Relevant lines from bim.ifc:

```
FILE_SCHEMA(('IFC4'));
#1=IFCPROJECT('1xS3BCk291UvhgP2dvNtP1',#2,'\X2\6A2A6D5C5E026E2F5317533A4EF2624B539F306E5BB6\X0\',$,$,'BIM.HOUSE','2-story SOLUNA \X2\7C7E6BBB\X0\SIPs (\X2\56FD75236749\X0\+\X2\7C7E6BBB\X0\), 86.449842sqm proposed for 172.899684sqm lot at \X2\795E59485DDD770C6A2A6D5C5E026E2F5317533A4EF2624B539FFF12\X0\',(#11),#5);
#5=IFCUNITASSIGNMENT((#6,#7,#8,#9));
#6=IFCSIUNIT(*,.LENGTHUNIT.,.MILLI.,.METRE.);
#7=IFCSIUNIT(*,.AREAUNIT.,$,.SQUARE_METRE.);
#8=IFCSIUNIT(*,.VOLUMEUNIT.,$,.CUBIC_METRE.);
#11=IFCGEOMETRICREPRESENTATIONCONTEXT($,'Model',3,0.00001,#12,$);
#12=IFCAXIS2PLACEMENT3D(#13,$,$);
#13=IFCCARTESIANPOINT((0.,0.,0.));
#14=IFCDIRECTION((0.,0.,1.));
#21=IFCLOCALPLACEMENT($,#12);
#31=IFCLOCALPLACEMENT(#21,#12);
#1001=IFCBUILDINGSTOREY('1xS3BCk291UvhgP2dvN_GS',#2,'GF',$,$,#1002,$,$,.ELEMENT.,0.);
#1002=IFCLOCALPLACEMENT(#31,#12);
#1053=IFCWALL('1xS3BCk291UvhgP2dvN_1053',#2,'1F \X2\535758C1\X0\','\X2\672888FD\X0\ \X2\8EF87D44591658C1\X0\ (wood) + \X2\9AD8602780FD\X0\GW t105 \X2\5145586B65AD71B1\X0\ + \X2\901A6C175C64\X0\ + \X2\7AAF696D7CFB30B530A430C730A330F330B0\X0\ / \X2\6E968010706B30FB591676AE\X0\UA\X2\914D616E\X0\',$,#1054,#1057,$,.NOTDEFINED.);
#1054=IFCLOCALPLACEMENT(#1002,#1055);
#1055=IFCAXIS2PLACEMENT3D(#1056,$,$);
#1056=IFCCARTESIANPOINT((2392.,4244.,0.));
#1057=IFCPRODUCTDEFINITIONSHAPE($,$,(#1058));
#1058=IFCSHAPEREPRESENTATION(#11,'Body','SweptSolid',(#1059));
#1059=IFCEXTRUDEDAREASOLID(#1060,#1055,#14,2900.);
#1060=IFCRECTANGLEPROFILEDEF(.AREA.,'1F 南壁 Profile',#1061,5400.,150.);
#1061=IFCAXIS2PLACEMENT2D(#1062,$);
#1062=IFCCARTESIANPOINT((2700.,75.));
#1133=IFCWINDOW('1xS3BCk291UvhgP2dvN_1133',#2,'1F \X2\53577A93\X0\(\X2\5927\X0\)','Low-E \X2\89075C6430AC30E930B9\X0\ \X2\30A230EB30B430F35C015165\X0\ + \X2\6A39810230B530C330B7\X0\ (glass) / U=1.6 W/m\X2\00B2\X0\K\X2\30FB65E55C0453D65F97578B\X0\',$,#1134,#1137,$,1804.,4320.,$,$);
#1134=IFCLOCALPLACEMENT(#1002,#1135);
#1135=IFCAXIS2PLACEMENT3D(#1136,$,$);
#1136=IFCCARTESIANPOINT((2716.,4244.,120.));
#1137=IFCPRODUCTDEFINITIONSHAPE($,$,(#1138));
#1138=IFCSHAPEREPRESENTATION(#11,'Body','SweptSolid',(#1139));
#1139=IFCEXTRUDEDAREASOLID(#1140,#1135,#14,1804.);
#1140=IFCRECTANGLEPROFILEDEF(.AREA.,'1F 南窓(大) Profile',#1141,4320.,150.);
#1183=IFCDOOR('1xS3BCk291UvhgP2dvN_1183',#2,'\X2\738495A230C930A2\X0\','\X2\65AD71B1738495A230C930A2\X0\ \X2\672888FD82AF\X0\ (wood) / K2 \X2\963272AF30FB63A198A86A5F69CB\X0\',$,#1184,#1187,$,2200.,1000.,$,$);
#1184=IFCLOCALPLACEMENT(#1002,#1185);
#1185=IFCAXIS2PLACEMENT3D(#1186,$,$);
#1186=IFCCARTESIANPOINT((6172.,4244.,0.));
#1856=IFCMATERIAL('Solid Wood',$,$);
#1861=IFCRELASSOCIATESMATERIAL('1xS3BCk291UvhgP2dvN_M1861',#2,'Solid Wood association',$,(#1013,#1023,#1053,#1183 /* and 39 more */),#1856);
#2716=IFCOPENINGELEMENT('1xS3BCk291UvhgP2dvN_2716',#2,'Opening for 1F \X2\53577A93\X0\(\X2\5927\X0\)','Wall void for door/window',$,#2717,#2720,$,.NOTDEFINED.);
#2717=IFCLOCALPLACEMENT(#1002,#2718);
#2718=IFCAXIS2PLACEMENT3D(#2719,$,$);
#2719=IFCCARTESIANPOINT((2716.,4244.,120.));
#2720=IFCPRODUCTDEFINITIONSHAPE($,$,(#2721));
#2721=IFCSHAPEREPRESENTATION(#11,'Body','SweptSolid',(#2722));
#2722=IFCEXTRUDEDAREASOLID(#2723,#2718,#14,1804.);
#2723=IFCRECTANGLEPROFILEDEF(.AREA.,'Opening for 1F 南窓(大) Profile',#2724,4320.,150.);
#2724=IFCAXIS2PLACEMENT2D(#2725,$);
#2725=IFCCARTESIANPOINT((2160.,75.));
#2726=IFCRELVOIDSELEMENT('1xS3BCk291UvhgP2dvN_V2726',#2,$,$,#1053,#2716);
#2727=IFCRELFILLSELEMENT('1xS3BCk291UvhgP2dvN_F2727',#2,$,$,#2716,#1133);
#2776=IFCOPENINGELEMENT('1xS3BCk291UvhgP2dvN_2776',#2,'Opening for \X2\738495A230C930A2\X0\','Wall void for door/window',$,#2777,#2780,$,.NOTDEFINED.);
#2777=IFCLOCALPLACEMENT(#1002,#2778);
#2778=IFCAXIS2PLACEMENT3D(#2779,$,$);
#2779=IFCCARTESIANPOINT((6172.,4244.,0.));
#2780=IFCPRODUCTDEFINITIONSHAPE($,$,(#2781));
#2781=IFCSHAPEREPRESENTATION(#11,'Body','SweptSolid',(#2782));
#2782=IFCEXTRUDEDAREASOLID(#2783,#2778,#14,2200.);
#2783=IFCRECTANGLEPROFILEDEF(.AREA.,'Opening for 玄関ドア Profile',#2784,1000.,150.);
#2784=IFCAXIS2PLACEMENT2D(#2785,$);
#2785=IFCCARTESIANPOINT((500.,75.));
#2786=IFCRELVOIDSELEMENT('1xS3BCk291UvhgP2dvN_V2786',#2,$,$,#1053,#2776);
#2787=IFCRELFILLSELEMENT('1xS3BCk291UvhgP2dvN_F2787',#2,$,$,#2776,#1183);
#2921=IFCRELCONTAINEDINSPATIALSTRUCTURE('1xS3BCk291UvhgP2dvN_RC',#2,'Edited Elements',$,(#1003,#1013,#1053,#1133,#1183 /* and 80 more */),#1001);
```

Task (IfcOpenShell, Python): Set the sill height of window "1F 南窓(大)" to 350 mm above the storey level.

```python
import numpy as np
import ifcopenshell
import ifcopenshell.api.geometry
import ifcopenshell.geom
import ifcopenshell.util.element
import ifcopenshell.util.placement
import ifcopenshell.util.shape
import ifcopenshell.util.unit

model = ifcopenshell.open("bim.ifc")
unit_scale = ifcopenshell.util.unit.calculate_unit_scale(model)

window = model.by_guid("1xS3BCk291UvhgP2dvN_1133")
opening = window.FillsVoids[0].RelatingOpeningElement
storey = ifcopenshell.util.element.get_container(window, ifc_class="IfcBuildingStorey")
level = ifcopenshell.util.placement.get_local_placement(storey.ObjectPlacement)[2, 3]

# The opening's origin need not be at the sill, so measure its lowest point.
shape = ifcopenshell.geom.create_shape(ifcopenshell.geom.settings(), opening)
bottom = ifcopenshell.util.shape.get_shape_bottom_elevation(shape, shape.geometry) / unit_scale
dz = level + 350.0 - bottom

shift = np.array([0.0, 0.0, dz])
# The window is not placed relative to its opening, so move both.
for product in (opening, window):
    matrix = ifcopenshell.util.placement.get_local_placement(product.ObjectPlacement)
    matrix[:3, 3] += shift
    ifcopenshell.api.geometry.edit_object_placement(model, product=product, matrix=matrix, is_si=False)

print(f"moved by {dz * unit_scale:+.3f} m")

model.write("bim_updated.ifc")
```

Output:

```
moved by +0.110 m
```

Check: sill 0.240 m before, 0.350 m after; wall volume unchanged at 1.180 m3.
